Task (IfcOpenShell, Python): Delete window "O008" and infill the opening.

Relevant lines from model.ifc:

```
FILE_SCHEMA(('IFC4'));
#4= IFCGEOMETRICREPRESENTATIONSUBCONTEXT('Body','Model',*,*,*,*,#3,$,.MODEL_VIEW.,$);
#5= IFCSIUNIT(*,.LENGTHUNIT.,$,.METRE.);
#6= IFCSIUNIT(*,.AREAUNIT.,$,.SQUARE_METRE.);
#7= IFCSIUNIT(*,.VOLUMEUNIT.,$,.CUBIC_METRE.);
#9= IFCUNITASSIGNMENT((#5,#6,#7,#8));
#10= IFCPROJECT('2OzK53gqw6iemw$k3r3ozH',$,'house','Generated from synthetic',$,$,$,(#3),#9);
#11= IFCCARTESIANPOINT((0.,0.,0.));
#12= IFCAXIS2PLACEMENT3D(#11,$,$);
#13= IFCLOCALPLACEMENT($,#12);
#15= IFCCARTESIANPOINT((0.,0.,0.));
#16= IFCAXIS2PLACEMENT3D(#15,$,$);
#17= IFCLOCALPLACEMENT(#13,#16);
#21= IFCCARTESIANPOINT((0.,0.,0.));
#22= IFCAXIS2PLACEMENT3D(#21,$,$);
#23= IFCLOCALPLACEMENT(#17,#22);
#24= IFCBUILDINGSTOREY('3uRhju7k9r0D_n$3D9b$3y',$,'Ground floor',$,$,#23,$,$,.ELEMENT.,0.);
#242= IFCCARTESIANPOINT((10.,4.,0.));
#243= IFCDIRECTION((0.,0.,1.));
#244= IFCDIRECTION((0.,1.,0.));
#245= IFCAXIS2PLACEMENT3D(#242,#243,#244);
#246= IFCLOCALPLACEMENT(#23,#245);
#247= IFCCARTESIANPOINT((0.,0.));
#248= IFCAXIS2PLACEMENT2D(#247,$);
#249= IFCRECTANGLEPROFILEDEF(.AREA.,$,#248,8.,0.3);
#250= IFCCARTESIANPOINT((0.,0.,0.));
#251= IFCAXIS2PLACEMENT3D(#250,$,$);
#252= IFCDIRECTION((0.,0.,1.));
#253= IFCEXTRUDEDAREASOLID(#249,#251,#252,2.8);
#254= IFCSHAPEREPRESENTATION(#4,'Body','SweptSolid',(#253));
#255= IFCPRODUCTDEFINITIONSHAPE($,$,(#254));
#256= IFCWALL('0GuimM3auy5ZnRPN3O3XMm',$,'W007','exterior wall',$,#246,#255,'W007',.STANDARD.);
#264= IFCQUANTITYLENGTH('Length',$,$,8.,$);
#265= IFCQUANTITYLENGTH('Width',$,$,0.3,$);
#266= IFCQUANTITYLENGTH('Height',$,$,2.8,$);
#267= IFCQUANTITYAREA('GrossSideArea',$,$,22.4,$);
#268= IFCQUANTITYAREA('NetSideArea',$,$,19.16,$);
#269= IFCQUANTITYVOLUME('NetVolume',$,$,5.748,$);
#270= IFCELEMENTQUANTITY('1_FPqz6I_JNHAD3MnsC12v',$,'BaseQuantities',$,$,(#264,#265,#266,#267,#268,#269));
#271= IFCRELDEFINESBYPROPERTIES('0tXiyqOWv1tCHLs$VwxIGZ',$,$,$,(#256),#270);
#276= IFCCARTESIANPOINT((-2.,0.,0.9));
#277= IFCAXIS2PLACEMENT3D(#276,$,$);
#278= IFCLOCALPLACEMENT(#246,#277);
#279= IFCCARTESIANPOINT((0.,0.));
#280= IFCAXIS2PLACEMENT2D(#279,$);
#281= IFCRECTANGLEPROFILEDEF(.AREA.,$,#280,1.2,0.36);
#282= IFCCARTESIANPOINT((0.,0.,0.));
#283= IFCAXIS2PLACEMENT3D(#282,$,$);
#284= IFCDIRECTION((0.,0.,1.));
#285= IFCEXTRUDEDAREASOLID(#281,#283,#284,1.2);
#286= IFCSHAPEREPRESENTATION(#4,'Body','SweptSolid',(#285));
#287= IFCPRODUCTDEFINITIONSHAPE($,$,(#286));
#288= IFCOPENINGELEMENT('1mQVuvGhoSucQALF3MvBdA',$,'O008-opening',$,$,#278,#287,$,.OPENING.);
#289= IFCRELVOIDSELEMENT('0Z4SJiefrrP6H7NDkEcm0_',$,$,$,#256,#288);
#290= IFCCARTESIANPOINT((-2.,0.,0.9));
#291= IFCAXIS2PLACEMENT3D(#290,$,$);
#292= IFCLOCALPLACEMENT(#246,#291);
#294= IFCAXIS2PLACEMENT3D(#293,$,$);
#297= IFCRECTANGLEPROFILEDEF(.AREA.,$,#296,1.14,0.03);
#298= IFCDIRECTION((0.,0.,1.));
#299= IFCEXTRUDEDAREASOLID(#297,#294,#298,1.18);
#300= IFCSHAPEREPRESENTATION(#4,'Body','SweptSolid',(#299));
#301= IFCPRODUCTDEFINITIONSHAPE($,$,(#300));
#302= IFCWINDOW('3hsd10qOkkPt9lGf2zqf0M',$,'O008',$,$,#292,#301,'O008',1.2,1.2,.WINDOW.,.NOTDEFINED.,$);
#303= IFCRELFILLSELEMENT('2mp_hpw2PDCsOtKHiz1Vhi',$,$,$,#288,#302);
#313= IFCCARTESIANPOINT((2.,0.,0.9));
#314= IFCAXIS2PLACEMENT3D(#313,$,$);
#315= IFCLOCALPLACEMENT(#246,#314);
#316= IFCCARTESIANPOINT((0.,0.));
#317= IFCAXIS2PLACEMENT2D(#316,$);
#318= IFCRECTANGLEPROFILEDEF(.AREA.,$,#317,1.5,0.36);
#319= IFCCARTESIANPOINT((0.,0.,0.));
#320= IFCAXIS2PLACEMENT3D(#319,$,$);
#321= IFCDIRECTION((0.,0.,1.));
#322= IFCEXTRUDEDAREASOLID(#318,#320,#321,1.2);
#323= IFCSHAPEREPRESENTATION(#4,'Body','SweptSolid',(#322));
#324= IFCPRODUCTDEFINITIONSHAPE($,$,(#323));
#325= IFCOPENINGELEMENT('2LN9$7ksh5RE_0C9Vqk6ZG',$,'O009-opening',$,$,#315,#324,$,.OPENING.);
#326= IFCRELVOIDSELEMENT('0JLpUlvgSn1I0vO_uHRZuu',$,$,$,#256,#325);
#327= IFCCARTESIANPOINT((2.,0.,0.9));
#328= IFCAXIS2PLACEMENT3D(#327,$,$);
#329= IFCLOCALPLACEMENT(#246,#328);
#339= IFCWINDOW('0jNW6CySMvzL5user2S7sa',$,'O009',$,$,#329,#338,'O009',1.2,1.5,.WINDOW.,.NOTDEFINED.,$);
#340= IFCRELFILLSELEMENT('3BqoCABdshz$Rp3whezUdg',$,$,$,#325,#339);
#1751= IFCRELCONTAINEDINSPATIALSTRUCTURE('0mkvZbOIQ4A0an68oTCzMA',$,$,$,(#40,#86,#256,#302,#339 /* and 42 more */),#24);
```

```python
import ifcopenshell
import ifcopenshell.api.feature
import ifcopenshell.api.pset
import ifcopenshell.api.root
import ifcopenshell.geom
import ifcopenshell.util.element
import ifcopenshell.util.shape
import ifcopenshell.util.unit

model = ifcopenshell.open("model.ifc")
area_scale = ifcopenshell.util.unit.calculate_unit_scale(model, "AREAUNIT")
volume_scale = ifcopenshell.util.unit.calculate_unit_scale(model, "VOLUMEUNIT")
settings = ifcopenshell.geom.settings()


def volume(element):
    """Net volume in cubic metres, openings subtracted."""
    shape = ifcopenshell.geom.create_shape(settings, element)
    return ifcopenshell.util.shape.get_volume(shape.geometry)


window = model.by_id(302)
opening = window.FillsVoids[0].RelatingOpeningElement
wall = opening.VoidsElements[0].RelatingBuildingElement
before = volume(wall)

ifcopenshell.api.root.remove_product(model, product=window)
ifcopenshell.api.feature.remove_feature(model, feature=opening)

after = volume(wall)
thickness = 0.3  # wall thickness in metres

# Update the wall's stored quantities.
qto = model.by_id(ifcopenshell.util.element.get_pset(wall, "BaseQuantities", should_inherit=False)["id"])
ifcopenshell.api.pset.edit_qto(model, qto=qto, properties={
    "NetSideArea": after / thickness / area_scale,
    "NetVolume": after / volume_scale,
})

print(f"wall volume {before:.3f} -> {after:.3f} m3")

model.write("model_updated.ifc")
```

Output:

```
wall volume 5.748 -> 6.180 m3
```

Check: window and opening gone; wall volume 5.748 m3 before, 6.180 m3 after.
